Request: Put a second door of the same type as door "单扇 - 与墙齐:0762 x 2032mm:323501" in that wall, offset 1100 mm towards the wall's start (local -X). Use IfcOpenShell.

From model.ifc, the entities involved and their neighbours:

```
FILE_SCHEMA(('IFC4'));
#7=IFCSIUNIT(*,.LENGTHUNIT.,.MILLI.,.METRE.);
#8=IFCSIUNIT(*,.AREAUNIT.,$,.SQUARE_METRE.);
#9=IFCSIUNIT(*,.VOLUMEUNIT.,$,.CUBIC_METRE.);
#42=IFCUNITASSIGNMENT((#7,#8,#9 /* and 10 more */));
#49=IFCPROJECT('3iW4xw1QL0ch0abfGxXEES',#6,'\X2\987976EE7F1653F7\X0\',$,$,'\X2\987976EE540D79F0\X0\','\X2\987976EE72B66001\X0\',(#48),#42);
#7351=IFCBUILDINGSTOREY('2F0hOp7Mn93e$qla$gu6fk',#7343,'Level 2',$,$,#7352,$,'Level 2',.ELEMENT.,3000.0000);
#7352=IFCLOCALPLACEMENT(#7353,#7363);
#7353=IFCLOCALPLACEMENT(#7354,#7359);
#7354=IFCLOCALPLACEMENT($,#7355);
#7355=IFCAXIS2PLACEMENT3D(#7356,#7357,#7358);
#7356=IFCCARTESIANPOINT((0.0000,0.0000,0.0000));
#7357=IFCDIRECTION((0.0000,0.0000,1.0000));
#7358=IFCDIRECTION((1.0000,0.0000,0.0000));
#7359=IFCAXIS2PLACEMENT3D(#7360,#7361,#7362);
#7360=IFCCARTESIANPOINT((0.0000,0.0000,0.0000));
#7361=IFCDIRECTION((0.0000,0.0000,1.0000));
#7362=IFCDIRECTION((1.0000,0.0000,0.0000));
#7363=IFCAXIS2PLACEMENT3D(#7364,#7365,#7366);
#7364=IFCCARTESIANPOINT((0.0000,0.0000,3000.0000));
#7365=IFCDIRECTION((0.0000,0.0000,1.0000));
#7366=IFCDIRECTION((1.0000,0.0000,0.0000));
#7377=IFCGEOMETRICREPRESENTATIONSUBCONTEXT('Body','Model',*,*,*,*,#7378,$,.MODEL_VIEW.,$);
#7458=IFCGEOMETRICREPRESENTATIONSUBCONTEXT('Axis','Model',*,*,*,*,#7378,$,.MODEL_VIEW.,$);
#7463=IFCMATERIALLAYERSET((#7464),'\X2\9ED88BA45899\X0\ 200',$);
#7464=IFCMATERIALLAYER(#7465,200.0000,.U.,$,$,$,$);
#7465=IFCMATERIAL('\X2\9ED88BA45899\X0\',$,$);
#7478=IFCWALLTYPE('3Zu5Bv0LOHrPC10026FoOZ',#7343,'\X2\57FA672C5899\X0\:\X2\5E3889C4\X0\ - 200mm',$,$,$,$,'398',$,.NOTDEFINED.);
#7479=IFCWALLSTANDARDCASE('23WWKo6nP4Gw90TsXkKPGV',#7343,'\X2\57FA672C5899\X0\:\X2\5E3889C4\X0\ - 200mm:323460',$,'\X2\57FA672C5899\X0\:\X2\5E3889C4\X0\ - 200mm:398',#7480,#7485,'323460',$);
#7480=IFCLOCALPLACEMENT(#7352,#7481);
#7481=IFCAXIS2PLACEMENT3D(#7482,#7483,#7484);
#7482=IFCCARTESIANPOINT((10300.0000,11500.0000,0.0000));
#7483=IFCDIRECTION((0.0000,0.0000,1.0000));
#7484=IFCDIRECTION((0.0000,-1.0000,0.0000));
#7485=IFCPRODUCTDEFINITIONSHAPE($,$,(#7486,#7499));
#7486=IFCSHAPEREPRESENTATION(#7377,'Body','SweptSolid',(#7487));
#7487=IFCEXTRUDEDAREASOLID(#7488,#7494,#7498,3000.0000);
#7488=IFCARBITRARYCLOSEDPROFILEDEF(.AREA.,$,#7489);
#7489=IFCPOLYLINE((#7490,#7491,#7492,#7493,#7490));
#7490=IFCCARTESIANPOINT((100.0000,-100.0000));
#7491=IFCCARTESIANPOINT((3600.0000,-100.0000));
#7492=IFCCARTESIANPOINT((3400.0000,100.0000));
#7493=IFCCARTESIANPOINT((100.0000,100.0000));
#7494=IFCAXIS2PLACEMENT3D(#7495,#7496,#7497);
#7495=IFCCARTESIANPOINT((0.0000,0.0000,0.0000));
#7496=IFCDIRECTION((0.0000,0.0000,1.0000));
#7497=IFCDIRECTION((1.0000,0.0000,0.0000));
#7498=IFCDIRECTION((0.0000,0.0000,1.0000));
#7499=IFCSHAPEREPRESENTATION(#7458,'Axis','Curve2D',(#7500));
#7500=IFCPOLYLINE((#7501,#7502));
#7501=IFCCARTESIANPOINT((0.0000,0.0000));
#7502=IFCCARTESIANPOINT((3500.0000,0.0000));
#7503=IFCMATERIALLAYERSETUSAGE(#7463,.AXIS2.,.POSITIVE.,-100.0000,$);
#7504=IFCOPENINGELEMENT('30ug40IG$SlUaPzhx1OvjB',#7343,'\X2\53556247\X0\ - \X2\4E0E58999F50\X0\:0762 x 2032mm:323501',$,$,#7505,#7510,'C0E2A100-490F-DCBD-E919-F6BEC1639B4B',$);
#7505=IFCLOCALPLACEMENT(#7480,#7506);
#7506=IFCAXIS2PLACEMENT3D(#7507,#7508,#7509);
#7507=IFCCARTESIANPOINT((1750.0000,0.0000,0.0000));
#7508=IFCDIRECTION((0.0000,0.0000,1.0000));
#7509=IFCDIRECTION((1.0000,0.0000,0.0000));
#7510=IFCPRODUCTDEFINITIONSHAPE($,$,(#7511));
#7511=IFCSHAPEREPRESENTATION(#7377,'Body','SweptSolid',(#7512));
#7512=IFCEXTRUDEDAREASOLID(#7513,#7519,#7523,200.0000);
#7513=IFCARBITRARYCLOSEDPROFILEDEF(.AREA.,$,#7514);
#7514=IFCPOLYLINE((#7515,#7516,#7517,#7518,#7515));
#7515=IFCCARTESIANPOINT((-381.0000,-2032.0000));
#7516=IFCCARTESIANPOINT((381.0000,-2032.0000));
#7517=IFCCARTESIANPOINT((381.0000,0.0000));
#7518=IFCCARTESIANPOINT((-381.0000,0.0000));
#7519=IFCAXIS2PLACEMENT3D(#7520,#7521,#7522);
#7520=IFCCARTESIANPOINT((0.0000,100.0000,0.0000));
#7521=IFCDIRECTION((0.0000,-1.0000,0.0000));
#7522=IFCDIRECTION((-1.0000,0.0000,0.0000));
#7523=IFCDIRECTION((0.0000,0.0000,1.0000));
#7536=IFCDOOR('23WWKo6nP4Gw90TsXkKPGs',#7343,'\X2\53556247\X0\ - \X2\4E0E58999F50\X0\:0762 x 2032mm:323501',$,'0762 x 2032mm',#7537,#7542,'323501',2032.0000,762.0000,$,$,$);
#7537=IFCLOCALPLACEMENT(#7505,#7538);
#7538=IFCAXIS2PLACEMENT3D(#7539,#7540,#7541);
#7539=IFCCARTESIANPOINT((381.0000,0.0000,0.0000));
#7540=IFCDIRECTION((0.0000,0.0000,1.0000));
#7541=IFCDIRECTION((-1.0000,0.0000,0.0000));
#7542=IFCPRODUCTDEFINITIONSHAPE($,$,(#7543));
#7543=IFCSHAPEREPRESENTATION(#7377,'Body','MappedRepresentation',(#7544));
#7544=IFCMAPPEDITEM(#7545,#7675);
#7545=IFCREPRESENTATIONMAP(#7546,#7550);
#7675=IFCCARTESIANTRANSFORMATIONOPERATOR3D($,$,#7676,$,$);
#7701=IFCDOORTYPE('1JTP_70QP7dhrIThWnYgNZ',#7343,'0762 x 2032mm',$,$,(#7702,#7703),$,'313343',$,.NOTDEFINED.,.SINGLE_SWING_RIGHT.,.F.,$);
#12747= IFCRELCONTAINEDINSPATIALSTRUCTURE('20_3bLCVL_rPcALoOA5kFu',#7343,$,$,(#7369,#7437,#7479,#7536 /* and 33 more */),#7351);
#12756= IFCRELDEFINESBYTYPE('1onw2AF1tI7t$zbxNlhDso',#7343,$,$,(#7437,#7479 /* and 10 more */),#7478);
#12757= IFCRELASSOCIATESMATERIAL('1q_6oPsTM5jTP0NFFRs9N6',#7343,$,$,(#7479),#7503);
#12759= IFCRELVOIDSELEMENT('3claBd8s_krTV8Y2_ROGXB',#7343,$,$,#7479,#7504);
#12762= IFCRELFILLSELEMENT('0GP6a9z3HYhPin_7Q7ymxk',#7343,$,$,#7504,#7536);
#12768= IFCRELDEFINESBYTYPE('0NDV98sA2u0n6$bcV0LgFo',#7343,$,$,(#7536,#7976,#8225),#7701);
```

```python
import ifcopenshell
import ifcopenshell.api.feature
import ifcopenshell.api.geometry
import ifcopenshell.api.root
import ifcopenshell.geom
import ifcopenshell.util.element
import ifcopenshell.util.placement
import ifcopenshell.util.shape

model = ifcopenshell.open("model.ifc")
settings = ifcopenshell.geom.settings()


def volume(element):
    """Net volume in cubic metres, openings subtracted."""
    shape = ifcopenshell.geom.create_shape(settings, element)
    return ifcopenshell.util.shape.get_volume(shape.geometry)


def reuse_history(source, copy):
    """copy_class also copies each property set's owner history, people and application; keep the originals."""
    for rel in copy.IsDefinedBy:
        if rel.is_a("IfcRelDefinesByProperties") and (history := rel.RelatingPropertyDefinition.OwnerHistory):
            rel.RelatingPropertyDefinition.OwnerHistory = source.OwnerHistory
            ifcopenshell.util.element.remove_deep2(model, history)


door = model.by_id(7536)
opening = door.FillsVoids[0].RelatingOpeningElement
wall = opening.VoidsElements[0].RelatingBuildingElement
before = volume(wall)
shift = ifcopenshell.util.placement.get_local_placement(wall.ObjectPlacement)[:3, 0] * -1100.0

# copy_class copies the void relationship, type, container and properties, but no geometry.
new_opening = ifcopenshell.api.root.copy_class(model, product=opening)
new_opening.Representation = ifcopenshell.util.element.copy_deep(
    model, opening.Representation, exclude=["IfcGeometricRepresentationContext", "IfcRepresentationMap"]
)
new_opening.Name = "单扇 - 与墙齐:0762 x 2032mm"
new_opening.Tag = None
new_door = ifcopenshell.api.root.copy_class(model, product=door)
new_door.Representation = ifcopenshell.util.element.copy_deep(
    model, door.Representation, exclude=["IfcGeometricRepresentationContext", "IfcRepresentationMap"]
)
new_door.Name = "单扇 - 与墙齐:0762 x 2032mm"
new_door.Tag = None
reuse_history(door, new_door)
ifcopenshell.api.feature.add_filling(model, opening=new_opening, element=new_door)

for old, new in ((opening, new_opening), (door, new_door)):
    matrix = ifcopenshell.util.placement.get_local_placement(old.ObjectPlacement)
    matrix[:3, 3] += shift
    ifcopenshell.api.geometry.edit_object_placement(model, product=new, matrix=matrix, is_si=False)

after = volume(wall)

print(f"wall volume {before:.3f} -> {after:.3f} m3")

model.write("model_rev.ifc")
```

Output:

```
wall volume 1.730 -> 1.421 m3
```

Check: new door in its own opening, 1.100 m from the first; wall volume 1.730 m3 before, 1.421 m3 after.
